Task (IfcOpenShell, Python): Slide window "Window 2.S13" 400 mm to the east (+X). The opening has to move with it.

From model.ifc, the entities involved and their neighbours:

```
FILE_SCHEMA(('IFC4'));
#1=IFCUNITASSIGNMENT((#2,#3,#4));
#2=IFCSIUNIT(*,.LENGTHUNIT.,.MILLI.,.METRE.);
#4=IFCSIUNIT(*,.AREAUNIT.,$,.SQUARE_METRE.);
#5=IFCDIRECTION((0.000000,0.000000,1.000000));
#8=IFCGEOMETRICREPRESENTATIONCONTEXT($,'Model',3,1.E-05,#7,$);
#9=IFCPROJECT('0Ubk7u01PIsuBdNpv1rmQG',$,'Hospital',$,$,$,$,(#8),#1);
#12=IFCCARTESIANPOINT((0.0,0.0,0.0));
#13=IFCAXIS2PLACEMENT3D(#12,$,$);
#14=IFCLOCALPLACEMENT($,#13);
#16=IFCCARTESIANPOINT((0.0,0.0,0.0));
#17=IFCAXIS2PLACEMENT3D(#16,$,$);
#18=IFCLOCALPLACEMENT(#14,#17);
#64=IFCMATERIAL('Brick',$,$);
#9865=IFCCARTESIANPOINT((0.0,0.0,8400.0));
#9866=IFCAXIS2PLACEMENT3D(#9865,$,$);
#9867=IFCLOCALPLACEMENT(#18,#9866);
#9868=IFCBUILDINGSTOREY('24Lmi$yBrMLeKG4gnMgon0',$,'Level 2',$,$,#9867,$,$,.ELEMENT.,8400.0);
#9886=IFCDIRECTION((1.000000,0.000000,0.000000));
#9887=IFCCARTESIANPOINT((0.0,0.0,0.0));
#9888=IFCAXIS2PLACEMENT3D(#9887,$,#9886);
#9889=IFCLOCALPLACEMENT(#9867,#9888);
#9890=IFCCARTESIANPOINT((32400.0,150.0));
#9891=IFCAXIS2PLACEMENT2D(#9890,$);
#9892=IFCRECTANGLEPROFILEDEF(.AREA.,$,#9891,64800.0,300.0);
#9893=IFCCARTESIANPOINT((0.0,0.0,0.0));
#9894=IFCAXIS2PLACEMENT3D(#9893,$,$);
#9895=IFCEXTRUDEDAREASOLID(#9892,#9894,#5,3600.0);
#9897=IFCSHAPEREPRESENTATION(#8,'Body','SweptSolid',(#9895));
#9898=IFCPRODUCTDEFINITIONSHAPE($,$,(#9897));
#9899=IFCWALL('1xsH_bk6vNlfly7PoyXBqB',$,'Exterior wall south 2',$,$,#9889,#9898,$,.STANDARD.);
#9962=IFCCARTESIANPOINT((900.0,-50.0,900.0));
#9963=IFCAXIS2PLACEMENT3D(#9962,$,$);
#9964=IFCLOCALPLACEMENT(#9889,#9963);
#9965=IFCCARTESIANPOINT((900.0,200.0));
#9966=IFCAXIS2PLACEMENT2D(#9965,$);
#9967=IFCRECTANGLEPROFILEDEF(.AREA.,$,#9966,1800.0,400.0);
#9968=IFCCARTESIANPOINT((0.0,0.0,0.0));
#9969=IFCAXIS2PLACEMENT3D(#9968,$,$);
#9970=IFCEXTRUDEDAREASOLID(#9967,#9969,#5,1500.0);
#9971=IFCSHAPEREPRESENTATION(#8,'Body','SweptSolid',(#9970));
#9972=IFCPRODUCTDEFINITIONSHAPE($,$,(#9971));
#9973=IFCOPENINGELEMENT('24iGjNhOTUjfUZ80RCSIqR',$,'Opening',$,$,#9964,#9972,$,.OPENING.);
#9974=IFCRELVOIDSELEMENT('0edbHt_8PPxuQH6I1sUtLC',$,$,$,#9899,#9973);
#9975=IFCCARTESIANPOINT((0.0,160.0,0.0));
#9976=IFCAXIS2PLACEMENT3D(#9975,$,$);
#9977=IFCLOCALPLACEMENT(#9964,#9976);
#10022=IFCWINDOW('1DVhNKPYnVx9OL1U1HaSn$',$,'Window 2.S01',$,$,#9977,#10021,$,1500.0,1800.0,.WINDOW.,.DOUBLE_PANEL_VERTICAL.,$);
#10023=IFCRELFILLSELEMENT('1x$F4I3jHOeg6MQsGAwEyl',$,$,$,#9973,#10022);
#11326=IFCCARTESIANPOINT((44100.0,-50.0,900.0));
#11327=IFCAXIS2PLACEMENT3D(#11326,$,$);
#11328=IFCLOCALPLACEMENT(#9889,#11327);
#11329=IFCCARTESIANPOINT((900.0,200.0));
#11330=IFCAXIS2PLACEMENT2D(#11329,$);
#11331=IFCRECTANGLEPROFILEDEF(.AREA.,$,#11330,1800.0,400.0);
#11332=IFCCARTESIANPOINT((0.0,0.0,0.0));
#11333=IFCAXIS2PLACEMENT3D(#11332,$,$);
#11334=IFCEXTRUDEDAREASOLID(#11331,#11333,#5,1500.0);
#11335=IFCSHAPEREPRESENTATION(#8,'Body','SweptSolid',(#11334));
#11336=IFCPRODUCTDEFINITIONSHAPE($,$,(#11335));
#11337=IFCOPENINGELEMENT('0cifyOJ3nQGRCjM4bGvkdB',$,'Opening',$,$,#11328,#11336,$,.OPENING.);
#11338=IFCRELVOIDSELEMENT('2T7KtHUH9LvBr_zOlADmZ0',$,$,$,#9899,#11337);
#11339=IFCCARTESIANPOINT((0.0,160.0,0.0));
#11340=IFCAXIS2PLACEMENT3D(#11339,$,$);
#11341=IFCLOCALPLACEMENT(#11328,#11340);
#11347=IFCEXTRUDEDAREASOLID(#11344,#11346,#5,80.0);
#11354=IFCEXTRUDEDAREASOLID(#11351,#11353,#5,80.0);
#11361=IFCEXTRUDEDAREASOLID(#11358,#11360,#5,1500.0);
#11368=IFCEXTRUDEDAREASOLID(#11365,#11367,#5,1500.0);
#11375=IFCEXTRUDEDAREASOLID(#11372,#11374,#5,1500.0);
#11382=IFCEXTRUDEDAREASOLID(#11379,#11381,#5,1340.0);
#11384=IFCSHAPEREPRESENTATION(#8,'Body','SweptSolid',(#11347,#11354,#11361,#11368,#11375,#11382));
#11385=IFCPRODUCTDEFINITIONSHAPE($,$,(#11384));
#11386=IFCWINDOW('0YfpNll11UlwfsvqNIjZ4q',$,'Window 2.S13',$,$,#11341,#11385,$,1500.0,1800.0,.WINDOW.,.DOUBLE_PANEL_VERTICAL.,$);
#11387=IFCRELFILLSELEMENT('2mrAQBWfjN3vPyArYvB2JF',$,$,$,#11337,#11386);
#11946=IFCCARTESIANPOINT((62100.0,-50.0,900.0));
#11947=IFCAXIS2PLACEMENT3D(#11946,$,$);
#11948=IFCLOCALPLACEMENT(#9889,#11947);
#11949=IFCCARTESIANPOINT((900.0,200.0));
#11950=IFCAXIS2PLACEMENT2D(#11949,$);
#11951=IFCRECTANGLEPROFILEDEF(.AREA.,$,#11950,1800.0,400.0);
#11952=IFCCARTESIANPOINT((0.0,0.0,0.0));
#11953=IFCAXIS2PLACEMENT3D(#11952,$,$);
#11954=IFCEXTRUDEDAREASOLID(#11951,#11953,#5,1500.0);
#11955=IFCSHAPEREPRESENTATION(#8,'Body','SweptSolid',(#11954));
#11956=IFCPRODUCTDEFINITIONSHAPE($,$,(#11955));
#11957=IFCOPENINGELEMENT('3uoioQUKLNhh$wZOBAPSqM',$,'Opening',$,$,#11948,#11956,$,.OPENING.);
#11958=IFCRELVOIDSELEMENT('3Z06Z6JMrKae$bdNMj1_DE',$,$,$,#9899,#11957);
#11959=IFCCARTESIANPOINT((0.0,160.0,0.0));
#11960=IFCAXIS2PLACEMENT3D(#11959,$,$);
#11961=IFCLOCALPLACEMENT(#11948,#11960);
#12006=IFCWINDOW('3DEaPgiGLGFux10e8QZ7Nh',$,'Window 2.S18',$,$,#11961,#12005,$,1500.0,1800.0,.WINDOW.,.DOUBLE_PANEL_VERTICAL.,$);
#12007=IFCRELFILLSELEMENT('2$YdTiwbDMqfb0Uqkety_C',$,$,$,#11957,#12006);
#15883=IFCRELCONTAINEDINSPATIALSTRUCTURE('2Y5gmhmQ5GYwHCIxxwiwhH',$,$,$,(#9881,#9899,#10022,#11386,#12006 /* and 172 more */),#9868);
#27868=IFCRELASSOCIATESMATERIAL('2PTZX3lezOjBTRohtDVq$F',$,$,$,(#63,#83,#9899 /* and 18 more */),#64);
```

```python
import ifcopenshell
import ifcopenshell.api.geometry
import ifcopenshell.util.placement

model = ifcopenshell.open("model.ifc")

window = model.by_guid("0YfpNll11UlwfsvqNIjZ4q")
opening = window.FillsVoids[0].RelatingOpeningElement
wall = opening.VoidsElements[0].RelatingBuildingElement

wall_matrix = ifcopenshell.util.placement.get_local_placement(wall.ObjectPlacement)
shift = wall_matrix[:3, 0] * 400.0
before = ifcopenshell.util.placement.get_local_placement(window.ObjectPlacement)[:3, 3].copy()

# The window is placed relative to its opening, so it follows when the opening moves.
matrix = ifcopenshell.util.placement.get_local_placement(opening.ObjectPlacement)
matrix[:3, 3] += shift
ifcopenshell.api.geometry.edit_object_placement(
    model, product=opening, matrix=matrix, is_si=False, should_transform_children=True
)

after = ifcopenshell.util.placement.get_local_placement(window.ObjectPlacement)[:3, 3]
print("window moved by", (after - before).round(3) + 0.0)

model.write("model_v2.ifc")
```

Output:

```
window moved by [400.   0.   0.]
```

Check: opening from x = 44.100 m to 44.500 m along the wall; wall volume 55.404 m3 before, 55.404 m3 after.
